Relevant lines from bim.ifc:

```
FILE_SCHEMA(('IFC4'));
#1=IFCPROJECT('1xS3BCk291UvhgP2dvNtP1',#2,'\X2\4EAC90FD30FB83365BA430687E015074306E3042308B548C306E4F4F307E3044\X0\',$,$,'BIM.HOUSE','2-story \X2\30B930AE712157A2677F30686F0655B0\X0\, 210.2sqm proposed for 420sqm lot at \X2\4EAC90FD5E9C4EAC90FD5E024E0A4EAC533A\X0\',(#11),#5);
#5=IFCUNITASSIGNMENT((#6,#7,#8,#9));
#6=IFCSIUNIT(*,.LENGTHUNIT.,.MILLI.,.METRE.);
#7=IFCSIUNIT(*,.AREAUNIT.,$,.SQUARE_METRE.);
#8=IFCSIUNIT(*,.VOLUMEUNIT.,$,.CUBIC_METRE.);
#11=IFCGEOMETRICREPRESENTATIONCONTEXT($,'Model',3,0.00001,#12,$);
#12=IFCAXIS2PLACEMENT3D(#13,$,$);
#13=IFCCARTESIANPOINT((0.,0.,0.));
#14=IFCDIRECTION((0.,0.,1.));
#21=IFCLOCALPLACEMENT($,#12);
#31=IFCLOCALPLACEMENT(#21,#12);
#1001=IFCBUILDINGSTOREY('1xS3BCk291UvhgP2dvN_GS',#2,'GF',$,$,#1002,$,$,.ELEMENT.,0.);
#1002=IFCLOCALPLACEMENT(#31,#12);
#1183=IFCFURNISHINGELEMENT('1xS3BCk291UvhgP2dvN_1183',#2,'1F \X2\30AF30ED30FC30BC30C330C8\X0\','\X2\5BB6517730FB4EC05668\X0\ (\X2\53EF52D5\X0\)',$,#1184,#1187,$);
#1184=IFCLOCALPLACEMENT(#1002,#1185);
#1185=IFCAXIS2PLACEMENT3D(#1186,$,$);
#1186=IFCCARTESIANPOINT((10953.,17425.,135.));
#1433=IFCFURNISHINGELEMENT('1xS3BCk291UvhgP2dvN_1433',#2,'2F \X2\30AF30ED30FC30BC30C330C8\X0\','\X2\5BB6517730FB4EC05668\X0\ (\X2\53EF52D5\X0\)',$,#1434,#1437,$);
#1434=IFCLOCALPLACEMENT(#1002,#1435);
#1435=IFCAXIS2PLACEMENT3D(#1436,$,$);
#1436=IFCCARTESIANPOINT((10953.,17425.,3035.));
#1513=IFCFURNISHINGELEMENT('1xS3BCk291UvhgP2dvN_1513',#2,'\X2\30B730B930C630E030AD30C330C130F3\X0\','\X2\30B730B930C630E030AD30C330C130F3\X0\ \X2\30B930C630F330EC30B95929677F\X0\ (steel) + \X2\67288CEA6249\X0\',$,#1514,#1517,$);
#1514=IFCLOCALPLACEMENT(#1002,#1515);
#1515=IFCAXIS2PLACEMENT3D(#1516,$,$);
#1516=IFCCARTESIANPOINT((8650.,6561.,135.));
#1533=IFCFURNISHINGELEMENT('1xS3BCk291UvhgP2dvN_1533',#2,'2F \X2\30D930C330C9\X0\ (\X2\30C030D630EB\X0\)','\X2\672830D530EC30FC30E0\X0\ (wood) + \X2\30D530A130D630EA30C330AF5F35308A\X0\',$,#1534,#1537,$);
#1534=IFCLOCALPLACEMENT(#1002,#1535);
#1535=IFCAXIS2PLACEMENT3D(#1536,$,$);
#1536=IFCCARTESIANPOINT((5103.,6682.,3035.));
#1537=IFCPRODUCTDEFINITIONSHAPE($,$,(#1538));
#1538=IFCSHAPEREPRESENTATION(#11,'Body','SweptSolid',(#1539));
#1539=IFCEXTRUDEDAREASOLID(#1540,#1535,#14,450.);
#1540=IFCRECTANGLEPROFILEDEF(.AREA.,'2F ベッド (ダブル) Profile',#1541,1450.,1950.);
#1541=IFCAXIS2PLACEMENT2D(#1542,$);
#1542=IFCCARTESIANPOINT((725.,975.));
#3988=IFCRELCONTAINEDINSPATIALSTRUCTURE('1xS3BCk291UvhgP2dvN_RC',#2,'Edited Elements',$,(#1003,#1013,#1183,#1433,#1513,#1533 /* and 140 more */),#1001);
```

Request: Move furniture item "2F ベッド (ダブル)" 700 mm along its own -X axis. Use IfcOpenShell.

```python
import ifcopenshell
import ifcopenshell.api.geometry
import ifcopenshell.util.placement

model = ifcopenshell.open("bim.ifc")

item = model.by_id(1533)
matrix = ifcopenshell.util.placement.get_local_placement(item.ObjectPlacement)
matrix[:3, 3] -= matrix[:3, 0] * 700.0
ifcopenshell.api.geometry.edit_object_placement(model, product=item, matrix=matrix, is_si=False)

print(ifcopenshell.util.placement.get_local_placement(item.ObjectPlacement).round(3) + 0.0)

model.write("bim_rev.ifc")
```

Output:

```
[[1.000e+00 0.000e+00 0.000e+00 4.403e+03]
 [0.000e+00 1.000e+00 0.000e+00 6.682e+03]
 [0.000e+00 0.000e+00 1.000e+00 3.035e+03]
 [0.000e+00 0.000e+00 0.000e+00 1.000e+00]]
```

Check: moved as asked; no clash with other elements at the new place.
